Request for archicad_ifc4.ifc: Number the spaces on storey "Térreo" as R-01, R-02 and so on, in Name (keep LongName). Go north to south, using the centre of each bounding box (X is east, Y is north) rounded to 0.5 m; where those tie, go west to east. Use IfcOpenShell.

First a look at what the model holds.

```python
import ifcopenshell
import ifcopenshell.util.element
import ifcopenshell.util.placement

model = ifcopenshell.open("archicad_ifc4.ifc")
print(model.schema)
storey = next(s for s in model.by_type("IfcBuildingStorey") if s.Name == "Térreo")
spaces = [e for e in ifcopenshell.util.element.get_decomposition(storey) if e.is_a("IfcSpace")]
for e in sorted(spaces, key=lambda e: e.id()):
    origin = ifcopenshell.util.placement.get_local_placement(e.ObjectPlacement)[:3, 3]
    print(e.id(), e.Name, e.LongName, origin.round(2) + 0.0, sep=" | ")
```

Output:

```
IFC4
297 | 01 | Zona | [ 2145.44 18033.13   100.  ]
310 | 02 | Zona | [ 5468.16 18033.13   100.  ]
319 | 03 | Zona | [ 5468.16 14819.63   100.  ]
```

```python
import ifcopenshell
import ifcopenshell.geom
import ifcopenshell.util.element
import ifcopenshell.util.shape

model = ifcopenshell.open("archicad_ifc4.ifc")
settings = ifcopenshell.geom.settings()
settings.set("use-world-coords", True)


def centre(element):
    shape = ifcopenshell.geom.create_shape(settings, element)
    return ifcopenshell.util.shape.get_bbox_centroid(shape.geometry)


storey = next(s for s in model.by_type("IfcBuildingStorey") if s.Name == "Térreo")
spaces = [e for e in ifcopenshell.util.element.get_decomposition(storey) if e.is_a("IfcSpace")]

# Insertion points can sit at a corner or the storey origin, so sort by the geometry (in metres).
centres = {e: centre(e) for e in spaces}
spaces.sort(key=lambda e: (-round(centres[e][1] / 0.5), centres[e][0]))

for i, e in enumerate(spaces, start=1):
    number = f"R-{i:02d}"
    e.Name = number
    print(e.id(), number)

model.write("archicad_ifc4_edited.ifc")
```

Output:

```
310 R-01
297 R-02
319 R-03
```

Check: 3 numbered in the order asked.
